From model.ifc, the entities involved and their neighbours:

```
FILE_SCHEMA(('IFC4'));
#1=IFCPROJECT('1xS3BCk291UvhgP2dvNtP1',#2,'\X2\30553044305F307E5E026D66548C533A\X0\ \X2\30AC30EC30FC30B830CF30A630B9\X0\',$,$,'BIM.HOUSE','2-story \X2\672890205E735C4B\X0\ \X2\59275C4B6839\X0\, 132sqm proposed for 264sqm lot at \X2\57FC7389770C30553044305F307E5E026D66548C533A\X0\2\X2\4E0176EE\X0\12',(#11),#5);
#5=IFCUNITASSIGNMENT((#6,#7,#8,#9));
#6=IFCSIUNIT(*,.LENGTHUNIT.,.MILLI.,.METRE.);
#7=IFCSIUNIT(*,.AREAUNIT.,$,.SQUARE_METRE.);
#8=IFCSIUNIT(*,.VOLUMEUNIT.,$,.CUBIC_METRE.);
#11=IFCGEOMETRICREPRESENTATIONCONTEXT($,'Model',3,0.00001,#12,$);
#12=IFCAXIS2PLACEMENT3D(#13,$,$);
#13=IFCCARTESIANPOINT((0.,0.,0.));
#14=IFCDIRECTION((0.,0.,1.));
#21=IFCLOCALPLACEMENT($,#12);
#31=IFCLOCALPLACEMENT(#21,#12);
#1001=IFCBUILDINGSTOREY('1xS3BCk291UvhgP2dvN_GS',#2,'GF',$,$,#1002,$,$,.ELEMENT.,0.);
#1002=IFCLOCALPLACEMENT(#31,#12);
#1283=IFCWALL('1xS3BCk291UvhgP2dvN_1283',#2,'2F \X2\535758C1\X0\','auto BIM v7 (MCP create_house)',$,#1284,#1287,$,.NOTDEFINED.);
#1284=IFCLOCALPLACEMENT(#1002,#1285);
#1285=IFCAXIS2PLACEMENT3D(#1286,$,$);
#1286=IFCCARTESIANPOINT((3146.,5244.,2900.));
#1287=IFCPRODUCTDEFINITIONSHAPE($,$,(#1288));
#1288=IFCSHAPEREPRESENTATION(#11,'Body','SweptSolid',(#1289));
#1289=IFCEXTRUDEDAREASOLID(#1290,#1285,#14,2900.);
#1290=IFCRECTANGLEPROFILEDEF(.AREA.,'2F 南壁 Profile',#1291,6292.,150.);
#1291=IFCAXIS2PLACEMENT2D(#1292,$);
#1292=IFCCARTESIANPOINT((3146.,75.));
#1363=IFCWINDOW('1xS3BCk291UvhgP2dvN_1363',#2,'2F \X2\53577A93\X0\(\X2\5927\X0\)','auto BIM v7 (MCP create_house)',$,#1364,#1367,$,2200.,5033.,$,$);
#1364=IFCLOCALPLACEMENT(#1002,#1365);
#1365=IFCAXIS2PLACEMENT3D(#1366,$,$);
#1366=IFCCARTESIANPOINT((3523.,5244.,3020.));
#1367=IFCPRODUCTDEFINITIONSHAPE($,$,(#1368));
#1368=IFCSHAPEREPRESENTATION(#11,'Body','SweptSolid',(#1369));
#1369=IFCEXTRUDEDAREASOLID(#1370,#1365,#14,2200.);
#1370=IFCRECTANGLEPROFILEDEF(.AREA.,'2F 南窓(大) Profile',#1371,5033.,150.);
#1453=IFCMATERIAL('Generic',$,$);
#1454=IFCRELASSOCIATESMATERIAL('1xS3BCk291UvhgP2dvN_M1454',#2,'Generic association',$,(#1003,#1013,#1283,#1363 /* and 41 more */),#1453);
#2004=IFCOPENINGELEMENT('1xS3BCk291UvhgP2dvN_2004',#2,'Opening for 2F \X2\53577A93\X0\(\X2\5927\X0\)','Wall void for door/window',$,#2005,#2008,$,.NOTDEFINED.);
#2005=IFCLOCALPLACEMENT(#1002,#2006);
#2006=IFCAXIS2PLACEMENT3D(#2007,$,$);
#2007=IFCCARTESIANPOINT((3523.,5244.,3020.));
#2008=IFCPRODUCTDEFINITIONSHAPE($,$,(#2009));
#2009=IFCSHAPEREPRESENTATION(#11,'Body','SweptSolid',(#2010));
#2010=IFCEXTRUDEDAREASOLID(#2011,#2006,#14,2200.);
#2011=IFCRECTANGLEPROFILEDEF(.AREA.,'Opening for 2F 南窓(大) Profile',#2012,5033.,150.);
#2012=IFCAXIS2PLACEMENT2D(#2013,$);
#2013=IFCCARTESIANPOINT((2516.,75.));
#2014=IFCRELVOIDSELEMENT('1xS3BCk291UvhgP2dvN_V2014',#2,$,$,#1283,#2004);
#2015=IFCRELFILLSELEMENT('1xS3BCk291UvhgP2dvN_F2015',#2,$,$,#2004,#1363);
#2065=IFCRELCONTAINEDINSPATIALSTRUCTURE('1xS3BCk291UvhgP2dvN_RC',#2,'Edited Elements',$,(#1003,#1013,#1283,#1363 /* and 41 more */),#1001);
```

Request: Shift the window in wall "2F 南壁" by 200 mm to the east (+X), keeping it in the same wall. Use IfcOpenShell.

```python
import ifcopenshell
import ifcopenshell.api.geometry
import ifcopenshell.util.placement

model = ifcopenshell.open("model.ifc")

window = model.by_guid("1xS3BCk291UvhgP2dvN_1363")
opening = window.FillsVoids[0].RelatingOpeningElement
wall = opening.VoidsElements[0].RelatingBuildingElement

wall_matrix = ifcopenshell.util.placement.get_local_placement(wall.ObjectPlacement)
shift = wall_matrix[:3, 0] * 200.0
before = ifcopenshell.util.placement.get_local_placement(window.ObjectPlacement)[:3, 3].copy()

# The window is not placed relative to its opening, so move both.
for product in (opening, window):
    matrix = ifcopenshell.util.placement.get_local_placement(product.ObjectPlacement)
    matrix[:3, 3] += shift
    ifcopenshell.api.geometry.edit_object_placement(model, product=product, matrix=matrix, is_si=False)

after = ifcopenshell.util.placement.get_local_placement(window.ObjectPlacement)[:3, 3]
print("window moved by", (after - before).round(3) + 0.0)

model.write("model_edited.ifc")
```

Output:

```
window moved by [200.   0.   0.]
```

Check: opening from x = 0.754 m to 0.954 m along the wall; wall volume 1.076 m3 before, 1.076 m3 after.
